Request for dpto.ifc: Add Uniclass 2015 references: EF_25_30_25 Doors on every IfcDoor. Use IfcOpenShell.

First a look at what the model holds.

```python
import ifcopenshell

model = ifcopenshell.open("dpto.ifc")
print(model.schema)
print("classifications:", [c.Name for c in model.by_type("IfcClassification")])
for ifc_class in ("IfcDoor", "IfcRoof", "IfcStair", "IfcWall", "IfcWindow"):
    print(ifc_class, len(model.by_type(ifc_class)))
```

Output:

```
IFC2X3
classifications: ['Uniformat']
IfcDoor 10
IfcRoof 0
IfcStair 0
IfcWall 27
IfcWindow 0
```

```python
import ifcopenshell
import ifcopenshell.api.classification

model = ifcopenshell.open("dpto.ifc")

# IFC2X3 requires Source and Edition and has no link from the project to the system.
system = model.create_entity("IfcClassification", Source="NBS", Edition="2015", Name="Uniclass 2015")

codes = {
    "IfcDoor": ("EF_25_30_25", "Doors"),
}
for ifc_class, (code, name) in codes.items():
    products = model.by_type(ifc_class)
    ifcopenshell.api.classification.add_reference(
        model, products=products, classification=system, identification=code, name=name
    )
    print(code, len(products))

model.write("dpto_v2.ifc")
```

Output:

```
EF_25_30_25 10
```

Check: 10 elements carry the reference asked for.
